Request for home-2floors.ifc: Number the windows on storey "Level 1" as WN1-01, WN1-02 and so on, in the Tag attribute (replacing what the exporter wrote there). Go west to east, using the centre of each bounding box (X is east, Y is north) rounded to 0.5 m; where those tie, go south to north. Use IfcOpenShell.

First a look at what the model holds.

```python
import ifcopenshell
import ifcopenshell.util.element
import ifcopenshell.util.placement

model = ifcopenshell.open("home-2floors.ifc")
print(model.schema)
storey = next(s for s in model.by_type("IfcBuildingStorey") if s.Name == "Level 1")
windows = [e for e in ifcopenshell.util.element.get_decomposition(storey) if e.is_a("IfcWindow")]
for e in sorted(windows, key=lambda e: e.id()):
    origin = ifcopenshell.util.placement.get_local_placement(e.ObjectPlacement)[:3, 3]
    print(e.id(), e.Tag, e.Name, origin.round(2) + 0.0, sep=" | ")
```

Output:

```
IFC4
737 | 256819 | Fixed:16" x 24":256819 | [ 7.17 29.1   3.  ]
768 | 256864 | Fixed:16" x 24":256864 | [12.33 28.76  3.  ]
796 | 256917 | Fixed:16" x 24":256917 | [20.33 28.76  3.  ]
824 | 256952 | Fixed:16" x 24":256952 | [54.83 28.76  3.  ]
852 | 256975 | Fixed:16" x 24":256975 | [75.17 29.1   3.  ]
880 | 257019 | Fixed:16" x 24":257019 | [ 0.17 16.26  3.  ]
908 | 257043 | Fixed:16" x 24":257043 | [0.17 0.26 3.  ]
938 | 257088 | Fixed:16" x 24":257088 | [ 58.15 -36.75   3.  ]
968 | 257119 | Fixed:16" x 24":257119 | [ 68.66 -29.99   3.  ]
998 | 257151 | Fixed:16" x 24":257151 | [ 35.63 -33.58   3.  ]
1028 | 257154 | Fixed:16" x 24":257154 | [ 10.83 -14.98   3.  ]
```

```python
import ifcopenshell
import ifcopenshell.geom
import ifcopenshell.util.element
import ifcopenshell.util.shape

model = ifcopenshell.open("home-2floors.ifc")
settings = ifcopenshell.geom.settings()
settings.set("use-world-coords", True)


def centre(element):
    shape = ifcopenshell.geom.create_shape(settings, element)
    return ifcopenshell.util.shape.get_bbox_centroid(shape.geometry)


storey = next(s for s in model.by_type("IfcBuildingStorey") if s.Name == "Level 1")
windows = [e for e in ifcopenshell.util.element.get_decomposition(storey) if e.is_a("IfcWindow")]

# Insertion points can sit at a corner or the storey origin, so sort by the geometry (in metres).
centres = {e: centre(e) for e in windows}
windows.sort(key=lambda e: (round(centres[e][0] / 0.5), centres[e][1]))

for i, e in enumerate(windows, start=1):
    number = f"WN1-{i:02d}"
    e.Tag = number
    print(e.id(), number)

model.write("home-2floors_rev.ifc")
```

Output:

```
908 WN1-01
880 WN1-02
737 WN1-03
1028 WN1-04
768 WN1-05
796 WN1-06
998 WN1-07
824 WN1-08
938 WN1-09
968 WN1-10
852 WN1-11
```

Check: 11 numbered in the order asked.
